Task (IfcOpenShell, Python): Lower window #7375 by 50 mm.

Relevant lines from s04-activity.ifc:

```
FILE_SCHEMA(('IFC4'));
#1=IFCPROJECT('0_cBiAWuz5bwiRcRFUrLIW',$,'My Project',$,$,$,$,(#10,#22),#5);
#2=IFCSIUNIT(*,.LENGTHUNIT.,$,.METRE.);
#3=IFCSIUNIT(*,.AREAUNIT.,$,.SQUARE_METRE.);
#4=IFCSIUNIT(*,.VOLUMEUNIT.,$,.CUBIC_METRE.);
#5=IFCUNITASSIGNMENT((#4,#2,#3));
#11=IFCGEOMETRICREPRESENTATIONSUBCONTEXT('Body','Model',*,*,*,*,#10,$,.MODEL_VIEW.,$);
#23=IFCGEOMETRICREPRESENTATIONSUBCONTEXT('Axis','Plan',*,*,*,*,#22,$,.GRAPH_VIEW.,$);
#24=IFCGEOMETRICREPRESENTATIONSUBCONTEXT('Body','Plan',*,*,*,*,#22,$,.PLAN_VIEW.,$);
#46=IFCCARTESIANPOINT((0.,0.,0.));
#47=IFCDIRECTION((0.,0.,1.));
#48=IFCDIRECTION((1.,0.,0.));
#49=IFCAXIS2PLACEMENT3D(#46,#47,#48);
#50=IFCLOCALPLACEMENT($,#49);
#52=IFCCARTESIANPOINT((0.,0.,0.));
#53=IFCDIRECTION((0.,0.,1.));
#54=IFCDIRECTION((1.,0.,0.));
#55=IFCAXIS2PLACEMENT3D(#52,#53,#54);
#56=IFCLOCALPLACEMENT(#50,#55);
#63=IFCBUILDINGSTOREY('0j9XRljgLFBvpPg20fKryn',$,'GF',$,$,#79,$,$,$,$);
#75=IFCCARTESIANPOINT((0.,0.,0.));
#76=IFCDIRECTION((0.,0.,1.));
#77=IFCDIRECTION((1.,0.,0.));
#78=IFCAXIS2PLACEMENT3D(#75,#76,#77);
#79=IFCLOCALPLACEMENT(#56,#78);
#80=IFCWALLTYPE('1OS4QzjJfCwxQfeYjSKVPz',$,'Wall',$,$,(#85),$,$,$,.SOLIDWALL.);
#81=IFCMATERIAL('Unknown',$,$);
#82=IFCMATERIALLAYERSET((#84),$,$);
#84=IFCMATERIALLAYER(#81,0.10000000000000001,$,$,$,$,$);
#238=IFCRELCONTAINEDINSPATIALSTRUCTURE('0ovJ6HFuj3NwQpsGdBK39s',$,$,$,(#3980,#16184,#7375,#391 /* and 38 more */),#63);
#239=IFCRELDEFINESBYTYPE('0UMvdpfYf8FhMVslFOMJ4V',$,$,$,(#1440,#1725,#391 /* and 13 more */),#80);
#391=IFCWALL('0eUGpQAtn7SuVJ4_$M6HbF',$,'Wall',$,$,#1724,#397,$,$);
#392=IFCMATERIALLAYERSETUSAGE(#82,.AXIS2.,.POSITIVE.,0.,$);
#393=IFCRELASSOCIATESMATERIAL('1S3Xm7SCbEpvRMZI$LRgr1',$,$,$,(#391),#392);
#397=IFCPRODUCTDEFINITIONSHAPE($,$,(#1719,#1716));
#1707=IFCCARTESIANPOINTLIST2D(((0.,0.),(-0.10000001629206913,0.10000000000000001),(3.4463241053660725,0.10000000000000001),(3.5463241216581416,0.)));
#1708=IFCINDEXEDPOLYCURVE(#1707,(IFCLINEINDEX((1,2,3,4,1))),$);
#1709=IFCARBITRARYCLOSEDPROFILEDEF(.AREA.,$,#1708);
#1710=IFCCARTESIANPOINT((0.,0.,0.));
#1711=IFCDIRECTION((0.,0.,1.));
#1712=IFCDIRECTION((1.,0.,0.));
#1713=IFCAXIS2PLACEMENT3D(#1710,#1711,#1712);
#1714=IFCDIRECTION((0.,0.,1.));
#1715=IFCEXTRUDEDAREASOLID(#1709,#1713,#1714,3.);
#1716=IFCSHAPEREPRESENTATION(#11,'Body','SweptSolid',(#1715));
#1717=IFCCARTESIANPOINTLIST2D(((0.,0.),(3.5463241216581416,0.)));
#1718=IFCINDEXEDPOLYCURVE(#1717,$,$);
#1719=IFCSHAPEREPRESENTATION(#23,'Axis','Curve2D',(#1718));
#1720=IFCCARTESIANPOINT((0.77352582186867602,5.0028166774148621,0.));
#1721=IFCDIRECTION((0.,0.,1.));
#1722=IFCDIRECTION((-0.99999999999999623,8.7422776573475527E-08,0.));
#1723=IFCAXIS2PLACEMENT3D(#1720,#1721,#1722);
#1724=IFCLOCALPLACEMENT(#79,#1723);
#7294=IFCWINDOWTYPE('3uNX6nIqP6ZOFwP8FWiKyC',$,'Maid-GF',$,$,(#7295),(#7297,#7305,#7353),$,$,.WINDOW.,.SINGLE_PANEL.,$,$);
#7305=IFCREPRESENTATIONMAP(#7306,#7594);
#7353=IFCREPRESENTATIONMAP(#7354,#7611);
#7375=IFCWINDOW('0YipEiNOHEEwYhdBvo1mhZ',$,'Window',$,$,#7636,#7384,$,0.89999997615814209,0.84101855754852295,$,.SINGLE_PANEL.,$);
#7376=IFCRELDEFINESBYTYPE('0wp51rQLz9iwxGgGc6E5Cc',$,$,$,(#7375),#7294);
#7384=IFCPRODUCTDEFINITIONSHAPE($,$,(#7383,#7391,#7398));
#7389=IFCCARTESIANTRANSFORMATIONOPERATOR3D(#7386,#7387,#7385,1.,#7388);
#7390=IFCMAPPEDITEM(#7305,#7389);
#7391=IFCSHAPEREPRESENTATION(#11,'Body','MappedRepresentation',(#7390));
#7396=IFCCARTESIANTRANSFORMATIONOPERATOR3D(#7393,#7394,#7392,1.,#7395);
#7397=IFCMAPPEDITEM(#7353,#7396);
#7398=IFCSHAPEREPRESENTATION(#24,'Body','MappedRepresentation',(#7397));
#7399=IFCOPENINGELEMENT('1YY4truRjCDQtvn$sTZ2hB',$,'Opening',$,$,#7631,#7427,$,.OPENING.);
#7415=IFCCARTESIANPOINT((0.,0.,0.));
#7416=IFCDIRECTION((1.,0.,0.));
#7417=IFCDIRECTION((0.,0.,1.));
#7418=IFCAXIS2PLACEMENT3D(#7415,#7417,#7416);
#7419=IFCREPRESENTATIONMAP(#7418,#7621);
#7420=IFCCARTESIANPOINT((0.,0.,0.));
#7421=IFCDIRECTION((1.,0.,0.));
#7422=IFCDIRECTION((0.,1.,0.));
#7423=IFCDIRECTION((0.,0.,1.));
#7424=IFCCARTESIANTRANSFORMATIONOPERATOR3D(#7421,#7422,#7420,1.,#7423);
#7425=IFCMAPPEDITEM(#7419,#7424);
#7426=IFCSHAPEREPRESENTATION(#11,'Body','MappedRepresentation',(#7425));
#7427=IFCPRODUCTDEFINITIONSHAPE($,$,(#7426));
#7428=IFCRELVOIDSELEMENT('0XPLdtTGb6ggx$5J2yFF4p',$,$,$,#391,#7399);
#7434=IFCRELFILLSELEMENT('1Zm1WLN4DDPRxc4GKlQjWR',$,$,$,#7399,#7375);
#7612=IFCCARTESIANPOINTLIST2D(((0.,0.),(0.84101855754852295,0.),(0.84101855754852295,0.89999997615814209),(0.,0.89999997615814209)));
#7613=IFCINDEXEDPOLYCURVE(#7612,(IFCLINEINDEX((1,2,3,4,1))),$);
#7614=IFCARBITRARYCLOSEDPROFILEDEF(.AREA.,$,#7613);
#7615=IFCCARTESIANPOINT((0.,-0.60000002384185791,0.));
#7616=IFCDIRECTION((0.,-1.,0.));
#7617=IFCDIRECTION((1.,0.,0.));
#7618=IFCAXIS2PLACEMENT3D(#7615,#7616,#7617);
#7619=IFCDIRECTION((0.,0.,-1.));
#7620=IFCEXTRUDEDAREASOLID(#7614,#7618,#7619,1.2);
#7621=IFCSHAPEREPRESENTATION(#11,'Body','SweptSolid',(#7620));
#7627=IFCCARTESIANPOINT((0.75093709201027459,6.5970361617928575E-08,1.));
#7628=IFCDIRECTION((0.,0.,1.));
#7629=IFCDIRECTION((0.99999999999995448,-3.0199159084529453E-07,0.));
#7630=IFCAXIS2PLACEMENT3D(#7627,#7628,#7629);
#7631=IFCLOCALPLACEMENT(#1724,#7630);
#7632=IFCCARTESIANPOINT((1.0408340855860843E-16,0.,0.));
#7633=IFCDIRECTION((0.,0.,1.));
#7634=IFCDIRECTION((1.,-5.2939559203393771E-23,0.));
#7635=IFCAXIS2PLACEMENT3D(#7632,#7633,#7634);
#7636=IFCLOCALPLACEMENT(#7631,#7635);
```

```python
import numpy as np
import ifcopenshell
import ifcopenshell.api.geometry
import ifcopenshell.util.placement
import ifcopenshell.util.unit

model = ifcopenshell.open("s04-activity.ifc")
unit_scale = ifcopenshell.util.unit.calculate_unit_scale(model)

window = model.by_guid("0YipEiNOHEEwYhdBvo1mhZ")
opening = window.FillsVoids[0].RelatingOpeningElement
dz = -0.05 / unit_scale

shift = np.array([0.0, 0.0, dz])
# The window is placed relative to its opening, so it follows when the opening moves.
matrix = ifcopenshell.util.placement.get_local_placement(opening.ObjectPlacement)
matrix[:3, 3] += shift
ifcopenshell.api.geometry.edit_object_placement(
    model, product=opening, matrix=matrix, is_si=False, should_transform_children=True
)

print(f"moved by {dz * unit_scale:+.3f} m")

model.write("s04-activity_rev.ifc")
```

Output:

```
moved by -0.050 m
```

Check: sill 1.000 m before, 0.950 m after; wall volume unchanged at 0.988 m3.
